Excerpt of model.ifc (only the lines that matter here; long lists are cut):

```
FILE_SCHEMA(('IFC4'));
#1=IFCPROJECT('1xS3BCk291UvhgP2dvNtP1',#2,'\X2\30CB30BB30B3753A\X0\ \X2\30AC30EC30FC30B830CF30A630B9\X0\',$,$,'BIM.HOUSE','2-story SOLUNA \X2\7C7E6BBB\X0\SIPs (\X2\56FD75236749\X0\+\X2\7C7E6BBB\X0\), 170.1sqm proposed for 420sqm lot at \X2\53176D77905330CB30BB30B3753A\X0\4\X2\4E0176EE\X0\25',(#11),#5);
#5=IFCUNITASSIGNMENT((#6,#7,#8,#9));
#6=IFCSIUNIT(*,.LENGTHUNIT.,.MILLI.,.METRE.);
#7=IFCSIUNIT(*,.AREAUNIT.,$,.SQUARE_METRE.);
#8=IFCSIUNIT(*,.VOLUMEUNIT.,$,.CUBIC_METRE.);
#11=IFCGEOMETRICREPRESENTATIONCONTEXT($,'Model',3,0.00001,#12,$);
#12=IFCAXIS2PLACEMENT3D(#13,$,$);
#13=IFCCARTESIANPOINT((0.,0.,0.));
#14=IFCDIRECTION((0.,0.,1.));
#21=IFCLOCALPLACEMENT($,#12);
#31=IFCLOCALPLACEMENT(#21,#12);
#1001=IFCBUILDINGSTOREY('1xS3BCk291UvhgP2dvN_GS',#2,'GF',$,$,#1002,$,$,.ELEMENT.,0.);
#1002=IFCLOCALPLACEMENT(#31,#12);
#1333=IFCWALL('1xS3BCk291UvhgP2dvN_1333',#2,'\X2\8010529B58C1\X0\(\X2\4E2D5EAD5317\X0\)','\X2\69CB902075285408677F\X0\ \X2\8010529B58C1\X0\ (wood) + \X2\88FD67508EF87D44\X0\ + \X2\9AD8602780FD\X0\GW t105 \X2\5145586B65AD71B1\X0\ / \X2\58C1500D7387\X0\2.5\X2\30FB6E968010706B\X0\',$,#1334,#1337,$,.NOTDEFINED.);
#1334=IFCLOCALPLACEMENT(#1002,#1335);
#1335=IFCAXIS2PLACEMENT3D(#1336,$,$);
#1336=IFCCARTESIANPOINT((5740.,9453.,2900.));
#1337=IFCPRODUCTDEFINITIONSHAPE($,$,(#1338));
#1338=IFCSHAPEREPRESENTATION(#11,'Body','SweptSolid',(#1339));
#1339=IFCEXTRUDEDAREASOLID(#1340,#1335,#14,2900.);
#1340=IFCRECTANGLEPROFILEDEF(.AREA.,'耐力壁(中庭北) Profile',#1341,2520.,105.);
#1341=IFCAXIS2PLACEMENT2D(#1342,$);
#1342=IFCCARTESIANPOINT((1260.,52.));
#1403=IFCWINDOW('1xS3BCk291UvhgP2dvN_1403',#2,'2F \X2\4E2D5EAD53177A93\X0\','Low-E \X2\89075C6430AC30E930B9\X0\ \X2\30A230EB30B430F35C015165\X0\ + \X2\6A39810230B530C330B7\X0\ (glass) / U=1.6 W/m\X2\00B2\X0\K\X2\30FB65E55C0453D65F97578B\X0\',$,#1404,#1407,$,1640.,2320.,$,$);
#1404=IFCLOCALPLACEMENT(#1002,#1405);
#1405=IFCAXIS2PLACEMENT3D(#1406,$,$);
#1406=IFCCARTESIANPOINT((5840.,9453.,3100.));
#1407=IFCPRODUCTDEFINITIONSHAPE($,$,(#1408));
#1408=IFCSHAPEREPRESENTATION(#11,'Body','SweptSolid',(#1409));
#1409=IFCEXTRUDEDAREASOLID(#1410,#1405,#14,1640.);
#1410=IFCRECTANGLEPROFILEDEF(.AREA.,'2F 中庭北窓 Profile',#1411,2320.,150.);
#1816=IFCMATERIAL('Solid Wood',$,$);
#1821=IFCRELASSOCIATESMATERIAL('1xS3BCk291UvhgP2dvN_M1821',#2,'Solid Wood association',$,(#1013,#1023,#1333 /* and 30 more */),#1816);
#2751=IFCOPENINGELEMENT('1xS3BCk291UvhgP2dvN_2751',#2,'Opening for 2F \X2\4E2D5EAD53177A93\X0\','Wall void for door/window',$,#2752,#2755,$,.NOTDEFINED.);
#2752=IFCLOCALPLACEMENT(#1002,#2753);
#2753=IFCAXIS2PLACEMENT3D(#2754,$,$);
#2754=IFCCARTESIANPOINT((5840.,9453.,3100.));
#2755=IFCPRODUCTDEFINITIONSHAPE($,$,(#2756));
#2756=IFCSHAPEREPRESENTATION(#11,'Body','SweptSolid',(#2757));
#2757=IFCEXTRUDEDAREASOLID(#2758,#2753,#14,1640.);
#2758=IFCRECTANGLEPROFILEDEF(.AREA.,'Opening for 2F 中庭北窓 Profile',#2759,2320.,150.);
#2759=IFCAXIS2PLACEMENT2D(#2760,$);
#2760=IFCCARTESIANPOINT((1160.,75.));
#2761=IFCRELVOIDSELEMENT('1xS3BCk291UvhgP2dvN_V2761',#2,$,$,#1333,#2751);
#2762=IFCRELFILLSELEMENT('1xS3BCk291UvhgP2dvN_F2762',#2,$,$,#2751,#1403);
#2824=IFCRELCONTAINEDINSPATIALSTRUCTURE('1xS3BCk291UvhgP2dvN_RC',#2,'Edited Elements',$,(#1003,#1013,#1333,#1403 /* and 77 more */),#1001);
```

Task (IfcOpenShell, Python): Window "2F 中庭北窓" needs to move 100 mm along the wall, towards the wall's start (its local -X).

```python
import ifcopenshell
import ifcopenshell.api.geometry
import ifcopenshell.util.placement

model = ifcopenshell.open("model.ifc")

window = model.by_id(1403)
opening = window.FillsVoids[0].RelatingOpeningElement
wall = opening.VoidsElements[0].RelatingBuildingElement

wall_matrix = ifcopenshell.util.placement.get_local_placement(wall.ObjectPlacement)
shift = wall_matrix[:3, 0] * -100.0
before = ifcopenshell.util.placement.get_local_placement(window.ObjectPlacement)[:3, 3].copy()

# The window is not placed relative to its opening, so move both.
for product in (opening, window):
    matrix = ifcopenshell.util.placement.get_local_placement(product.ObjectPlacement)
    matrix[:3, 3] += shift
    ifcopenshell.api.geometry.edit_object_placement(model, product=product, matrix=matrix, is_si=False)

after = ifcopenshell.util.placement.get_local_placement(window.ObjectPlacement)[:3, 3]
print("window moved by", (after - before).round(3) + 0.0)

model.write("model_rev.ifc")
```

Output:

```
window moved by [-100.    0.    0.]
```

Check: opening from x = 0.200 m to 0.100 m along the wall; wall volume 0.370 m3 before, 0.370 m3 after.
